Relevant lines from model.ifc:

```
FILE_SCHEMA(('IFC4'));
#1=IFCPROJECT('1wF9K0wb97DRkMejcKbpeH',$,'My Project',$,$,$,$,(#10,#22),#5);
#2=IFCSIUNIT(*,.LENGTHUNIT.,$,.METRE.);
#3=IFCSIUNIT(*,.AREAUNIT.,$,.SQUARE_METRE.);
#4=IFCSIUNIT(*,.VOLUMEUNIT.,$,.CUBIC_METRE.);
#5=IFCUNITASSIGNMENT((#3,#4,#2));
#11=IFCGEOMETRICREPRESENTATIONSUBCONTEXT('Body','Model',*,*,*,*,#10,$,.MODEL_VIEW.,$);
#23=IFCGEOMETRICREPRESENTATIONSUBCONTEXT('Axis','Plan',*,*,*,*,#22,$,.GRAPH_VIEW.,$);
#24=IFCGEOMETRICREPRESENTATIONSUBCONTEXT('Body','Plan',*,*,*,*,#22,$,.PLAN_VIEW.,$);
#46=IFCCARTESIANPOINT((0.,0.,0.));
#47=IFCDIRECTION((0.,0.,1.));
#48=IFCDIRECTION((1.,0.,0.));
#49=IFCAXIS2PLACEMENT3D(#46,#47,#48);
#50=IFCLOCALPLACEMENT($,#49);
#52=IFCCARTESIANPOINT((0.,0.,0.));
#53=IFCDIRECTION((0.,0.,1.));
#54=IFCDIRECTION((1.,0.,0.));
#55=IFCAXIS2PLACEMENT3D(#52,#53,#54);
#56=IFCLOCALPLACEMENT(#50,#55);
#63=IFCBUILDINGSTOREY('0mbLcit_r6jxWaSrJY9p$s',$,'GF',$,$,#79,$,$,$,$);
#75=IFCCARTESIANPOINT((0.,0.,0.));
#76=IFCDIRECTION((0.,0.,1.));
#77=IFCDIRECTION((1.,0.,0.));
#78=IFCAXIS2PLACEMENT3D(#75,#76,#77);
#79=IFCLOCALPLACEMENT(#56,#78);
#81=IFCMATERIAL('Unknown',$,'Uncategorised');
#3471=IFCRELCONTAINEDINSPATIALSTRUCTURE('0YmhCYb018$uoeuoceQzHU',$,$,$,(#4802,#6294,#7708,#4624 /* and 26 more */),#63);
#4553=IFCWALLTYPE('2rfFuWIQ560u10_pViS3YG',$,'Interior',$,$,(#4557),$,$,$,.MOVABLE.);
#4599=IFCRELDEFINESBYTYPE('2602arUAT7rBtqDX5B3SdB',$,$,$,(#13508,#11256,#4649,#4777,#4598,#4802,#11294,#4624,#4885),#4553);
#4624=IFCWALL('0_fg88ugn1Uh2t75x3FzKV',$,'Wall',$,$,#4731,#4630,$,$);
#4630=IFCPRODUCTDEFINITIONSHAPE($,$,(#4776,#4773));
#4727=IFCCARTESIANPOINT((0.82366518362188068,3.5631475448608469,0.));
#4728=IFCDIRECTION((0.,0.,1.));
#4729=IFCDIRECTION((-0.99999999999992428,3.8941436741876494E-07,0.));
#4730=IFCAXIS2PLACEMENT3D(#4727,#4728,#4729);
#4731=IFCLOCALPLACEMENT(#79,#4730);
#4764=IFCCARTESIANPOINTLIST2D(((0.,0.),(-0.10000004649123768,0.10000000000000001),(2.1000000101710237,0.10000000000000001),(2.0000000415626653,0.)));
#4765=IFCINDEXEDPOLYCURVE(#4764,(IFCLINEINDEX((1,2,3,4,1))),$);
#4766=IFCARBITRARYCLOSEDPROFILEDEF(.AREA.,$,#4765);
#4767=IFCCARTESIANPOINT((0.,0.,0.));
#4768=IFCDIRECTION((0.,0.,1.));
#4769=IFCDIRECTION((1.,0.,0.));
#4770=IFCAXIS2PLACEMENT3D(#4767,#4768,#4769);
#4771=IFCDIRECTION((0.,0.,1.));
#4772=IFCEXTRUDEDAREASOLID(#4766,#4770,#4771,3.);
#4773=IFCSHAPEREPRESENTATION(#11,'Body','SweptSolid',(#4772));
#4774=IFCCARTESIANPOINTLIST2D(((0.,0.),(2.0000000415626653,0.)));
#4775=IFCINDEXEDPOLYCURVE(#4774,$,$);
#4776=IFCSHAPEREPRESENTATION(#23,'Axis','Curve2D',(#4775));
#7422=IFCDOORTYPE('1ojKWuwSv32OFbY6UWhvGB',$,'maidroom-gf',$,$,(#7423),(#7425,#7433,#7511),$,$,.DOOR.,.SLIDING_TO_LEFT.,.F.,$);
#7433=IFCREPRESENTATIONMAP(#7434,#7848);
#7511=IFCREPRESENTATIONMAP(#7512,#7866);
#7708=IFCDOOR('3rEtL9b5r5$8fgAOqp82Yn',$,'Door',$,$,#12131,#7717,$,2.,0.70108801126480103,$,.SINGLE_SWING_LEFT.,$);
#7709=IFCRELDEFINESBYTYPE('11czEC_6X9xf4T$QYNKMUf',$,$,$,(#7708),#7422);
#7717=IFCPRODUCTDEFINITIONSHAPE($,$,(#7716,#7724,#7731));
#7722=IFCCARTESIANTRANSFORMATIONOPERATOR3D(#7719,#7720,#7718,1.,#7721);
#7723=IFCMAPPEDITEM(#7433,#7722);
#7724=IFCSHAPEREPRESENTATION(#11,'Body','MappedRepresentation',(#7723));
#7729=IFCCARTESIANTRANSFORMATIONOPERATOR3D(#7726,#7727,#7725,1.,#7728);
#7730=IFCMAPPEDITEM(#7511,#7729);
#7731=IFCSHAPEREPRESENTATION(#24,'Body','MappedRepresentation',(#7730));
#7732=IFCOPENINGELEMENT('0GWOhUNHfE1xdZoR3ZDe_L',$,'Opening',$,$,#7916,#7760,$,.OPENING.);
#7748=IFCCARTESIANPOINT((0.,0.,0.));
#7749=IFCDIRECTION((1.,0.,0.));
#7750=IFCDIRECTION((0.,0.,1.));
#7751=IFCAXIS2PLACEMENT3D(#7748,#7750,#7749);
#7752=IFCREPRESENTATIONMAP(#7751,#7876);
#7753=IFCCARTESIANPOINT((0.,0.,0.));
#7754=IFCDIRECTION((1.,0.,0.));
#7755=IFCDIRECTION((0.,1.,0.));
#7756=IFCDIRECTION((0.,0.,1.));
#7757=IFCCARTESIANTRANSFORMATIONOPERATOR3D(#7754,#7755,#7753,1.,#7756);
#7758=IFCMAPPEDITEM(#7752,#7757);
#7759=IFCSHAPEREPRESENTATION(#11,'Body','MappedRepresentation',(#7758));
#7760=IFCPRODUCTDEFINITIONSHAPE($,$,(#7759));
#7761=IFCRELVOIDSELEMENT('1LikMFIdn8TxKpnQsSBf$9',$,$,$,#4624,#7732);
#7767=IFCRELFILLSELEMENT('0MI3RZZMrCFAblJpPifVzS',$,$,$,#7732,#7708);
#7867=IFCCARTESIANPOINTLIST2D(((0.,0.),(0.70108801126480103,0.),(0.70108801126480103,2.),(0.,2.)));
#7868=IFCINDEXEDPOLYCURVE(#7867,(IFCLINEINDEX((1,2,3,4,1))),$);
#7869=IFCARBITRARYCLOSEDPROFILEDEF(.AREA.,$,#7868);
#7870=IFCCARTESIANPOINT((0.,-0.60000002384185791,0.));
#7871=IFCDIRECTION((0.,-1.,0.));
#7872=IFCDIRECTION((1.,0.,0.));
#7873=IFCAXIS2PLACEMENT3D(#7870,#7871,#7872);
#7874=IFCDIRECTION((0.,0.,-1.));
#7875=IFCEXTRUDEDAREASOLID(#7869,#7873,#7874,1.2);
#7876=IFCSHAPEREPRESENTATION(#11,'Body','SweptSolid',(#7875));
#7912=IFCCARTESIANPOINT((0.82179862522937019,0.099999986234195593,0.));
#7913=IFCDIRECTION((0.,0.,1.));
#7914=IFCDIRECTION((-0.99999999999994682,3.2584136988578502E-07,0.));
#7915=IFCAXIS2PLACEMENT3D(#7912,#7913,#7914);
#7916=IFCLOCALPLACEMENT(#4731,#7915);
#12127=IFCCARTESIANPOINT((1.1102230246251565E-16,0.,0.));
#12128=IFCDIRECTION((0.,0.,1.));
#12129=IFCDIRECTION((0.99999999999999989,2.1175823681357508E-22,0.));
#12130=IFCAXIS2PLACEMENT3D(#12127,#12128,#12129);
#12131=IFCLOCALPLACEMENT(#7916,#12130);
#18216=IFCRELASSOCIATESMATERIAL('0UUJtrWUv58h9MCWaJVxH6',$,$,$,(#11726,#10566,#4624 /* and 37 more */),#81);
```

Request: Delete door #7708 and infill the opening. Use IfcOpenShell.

```python
import ifcopenshell
import ifcopenshell.api.feature
import ifcopenshell.api.root
import ifcopenshell.geom
import ifcopenshell.util.shape

model = ifcopenshell.open("model.ifc")
settings = ifcopenshell.geom.settings()


def volume(element):
    """Net volume in cubic metres, openings subtracted."""
    shape = ifcopenshell.geom.create_shape(settings, element)
    return ifcopenshell.util.shape.get_volume(shape.geometry)


door = model.by_guid("3rEtL9b5r5$8fgAOqp82Yn")
opening = door.FillsVoids[0].RelatingOpeningElement
wall = opening.VoidsElements[0].RelatingBuildingElement
before = volume(wall)

ifcopenshell.api.root.remove_product(model, product=door)
ifcopenshell.api.feature.remove_feature(model, feature=opening)

after = volume(wall)

print(f"wall volume {before:.3f} -> {after:.3f} m3")

model.write("model_updated.ifc")
```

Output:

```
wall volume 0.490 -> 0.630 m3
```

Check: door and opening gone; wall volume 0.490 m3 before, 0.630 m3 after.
